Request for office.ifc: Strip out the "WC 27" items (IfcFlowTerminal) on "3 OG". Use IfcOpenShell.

First a look at what the model holds.

```python
import ifcopenshell
import ifcopenshell.util.element

model = ifcopenshell.open("office.ifc")
print(model.schema)
storey = next(s for s in model.by_type("IfcBuildingStorey") if s.Name == "3 OG")
terminals = [e for e in ifcopenshell.util.element.get_decomposition(storey) if e.is_a("IfcFlowTerminal")]
seen = {}
for e in terminals:
    element_type = ifcopenshell.util.element.get_type(e)
    name = element_type.Name if element_type not in (None, e) else None
    seen[name] = seen.get(name, 0) + 1
for name, count in sorted(seen.items(), key=str):
    print(count, "x", name)
```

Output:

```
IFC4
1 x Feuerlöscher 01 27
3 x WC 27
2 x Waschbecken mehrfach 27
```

```python
import ifcopenshell
import ifcopenshell.api.root
import ifcopenshell.util.element

model = ifcopenshell.open("office.ifc")

storey = next(s for s in model.by_type("IfcBuildingStorey") if s.Name == "3 OG")
terminals = [e for e in ifcopenshell.util.element.get_decomposition(storey) if e.is_a("IfcFlowTerminal")]
targets = [e for e in terminals if (t := ifcopenshell.util.element.get_type(e)) not in (None, e) and t.Name == "WC 27"]

for e in targets:
    ifcopenshell.api.root.remove_product(model, product=e)
print(len(targets), "removed")

model.write("office-out.ifc")
```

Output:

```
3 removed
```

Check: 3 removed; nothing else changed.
